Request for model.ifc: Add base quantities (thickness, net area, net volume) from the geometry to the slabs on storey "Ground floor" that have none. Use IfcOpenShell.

First a look at what the model holds.

```python
import ifcopenshell
import ifcopenshell.util.element
import ifcopenshell.util.unit

model = ifcopenshell.open("model.ifc")
print(model.schema)
for unit_type in ("LENGTHUNIT", "AREAUNIT", "VOLUMEUNIT"):
    print(unit_type, ifcopenshell.util.unit.calculate_unit_scale(model, unit_type))
storey = next(s for s in model.by_type("IfcBuildingStorey") if s.Name == "Ground floor")
slabs = [e for e in ifcopenshell.util.element.get_decomposition(storey) if e.is_a("IfcSlab")]
for e in sorted(slabs, key=lambda e: e.id()):
    print(e.id(), e.is_a(), e.Name, list(ifcopenshell.util.element.get_psets(e, qtos_only=True)), sep=" | ")
```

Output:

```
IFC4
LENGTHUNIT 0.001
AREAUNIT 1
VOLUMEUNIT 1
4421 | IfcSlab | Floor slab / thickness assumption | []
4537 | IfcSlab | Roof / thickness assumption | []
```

```python
import ifcopenshell
import ifcopenshell.api.pset
import ifcopenshell.geom
import ifcopenshell.util.element
import ifcopenshell.util.shape
import ifcopenshell.util.unit

model = ifcopenshell.open("model.ifc")
unit_scale = ifcopenshell.util.unit.calculate_unit_scale(model)
area_scale = ifcopenshell.util.unit.calculate_unit_scale(model, "AREAUNIT")
volume_scale = ifcopenshell.util.unit.calculate_unit_scale(model, "VOLUMEUNIT")
settings = ifcopenshell.geom.settings()

storey = next(s for s in model.by_type("IfcBuildingStorey") if s.Name == "Ground floor")
slabs = [e for e in ifcopenshell.util.element.get_decomposition(storey) if e.is_a("IfcSlab")]

for e in sorted(slabs, key=lambda e: e.id()):
    if ifcopenshell.util.element.get_psets(e, qtos_only=True, should_inherit=False):
        continue
    # Geometry comes back in metres, in the element's own axes.
    shape = ifcopenshell.geom.create_shape(settings, e)
    values = {
        "Width": ifcopenshell.util.shape.get_z(shape.geometry) / unit_scale,
        "NetArea": ifcopenshell.util.shape.get_footprint_area(shape.geometry) / area_scale,
        "NetVolume": ifcopenshell.util.shape.get_volume(shape.geometry) / volume_scale,
    }
    qto = ifcopenshell.api.pset.add_qto(model, product=e, name="Qto_SlabBaseQuantities")
    ifcopenshell.api.pset.edit_qto(model, qto=qto, properties=values)
    print(e.id(), {k: round(v, 3) for k, v in values.items()})

model.write("model_v2.ifc")
```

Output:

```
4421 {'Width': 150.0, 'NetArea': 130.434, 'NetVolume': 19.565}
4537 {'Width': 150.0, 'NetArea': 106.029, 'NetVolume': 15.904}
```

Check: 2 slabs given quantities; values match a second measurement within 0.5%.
